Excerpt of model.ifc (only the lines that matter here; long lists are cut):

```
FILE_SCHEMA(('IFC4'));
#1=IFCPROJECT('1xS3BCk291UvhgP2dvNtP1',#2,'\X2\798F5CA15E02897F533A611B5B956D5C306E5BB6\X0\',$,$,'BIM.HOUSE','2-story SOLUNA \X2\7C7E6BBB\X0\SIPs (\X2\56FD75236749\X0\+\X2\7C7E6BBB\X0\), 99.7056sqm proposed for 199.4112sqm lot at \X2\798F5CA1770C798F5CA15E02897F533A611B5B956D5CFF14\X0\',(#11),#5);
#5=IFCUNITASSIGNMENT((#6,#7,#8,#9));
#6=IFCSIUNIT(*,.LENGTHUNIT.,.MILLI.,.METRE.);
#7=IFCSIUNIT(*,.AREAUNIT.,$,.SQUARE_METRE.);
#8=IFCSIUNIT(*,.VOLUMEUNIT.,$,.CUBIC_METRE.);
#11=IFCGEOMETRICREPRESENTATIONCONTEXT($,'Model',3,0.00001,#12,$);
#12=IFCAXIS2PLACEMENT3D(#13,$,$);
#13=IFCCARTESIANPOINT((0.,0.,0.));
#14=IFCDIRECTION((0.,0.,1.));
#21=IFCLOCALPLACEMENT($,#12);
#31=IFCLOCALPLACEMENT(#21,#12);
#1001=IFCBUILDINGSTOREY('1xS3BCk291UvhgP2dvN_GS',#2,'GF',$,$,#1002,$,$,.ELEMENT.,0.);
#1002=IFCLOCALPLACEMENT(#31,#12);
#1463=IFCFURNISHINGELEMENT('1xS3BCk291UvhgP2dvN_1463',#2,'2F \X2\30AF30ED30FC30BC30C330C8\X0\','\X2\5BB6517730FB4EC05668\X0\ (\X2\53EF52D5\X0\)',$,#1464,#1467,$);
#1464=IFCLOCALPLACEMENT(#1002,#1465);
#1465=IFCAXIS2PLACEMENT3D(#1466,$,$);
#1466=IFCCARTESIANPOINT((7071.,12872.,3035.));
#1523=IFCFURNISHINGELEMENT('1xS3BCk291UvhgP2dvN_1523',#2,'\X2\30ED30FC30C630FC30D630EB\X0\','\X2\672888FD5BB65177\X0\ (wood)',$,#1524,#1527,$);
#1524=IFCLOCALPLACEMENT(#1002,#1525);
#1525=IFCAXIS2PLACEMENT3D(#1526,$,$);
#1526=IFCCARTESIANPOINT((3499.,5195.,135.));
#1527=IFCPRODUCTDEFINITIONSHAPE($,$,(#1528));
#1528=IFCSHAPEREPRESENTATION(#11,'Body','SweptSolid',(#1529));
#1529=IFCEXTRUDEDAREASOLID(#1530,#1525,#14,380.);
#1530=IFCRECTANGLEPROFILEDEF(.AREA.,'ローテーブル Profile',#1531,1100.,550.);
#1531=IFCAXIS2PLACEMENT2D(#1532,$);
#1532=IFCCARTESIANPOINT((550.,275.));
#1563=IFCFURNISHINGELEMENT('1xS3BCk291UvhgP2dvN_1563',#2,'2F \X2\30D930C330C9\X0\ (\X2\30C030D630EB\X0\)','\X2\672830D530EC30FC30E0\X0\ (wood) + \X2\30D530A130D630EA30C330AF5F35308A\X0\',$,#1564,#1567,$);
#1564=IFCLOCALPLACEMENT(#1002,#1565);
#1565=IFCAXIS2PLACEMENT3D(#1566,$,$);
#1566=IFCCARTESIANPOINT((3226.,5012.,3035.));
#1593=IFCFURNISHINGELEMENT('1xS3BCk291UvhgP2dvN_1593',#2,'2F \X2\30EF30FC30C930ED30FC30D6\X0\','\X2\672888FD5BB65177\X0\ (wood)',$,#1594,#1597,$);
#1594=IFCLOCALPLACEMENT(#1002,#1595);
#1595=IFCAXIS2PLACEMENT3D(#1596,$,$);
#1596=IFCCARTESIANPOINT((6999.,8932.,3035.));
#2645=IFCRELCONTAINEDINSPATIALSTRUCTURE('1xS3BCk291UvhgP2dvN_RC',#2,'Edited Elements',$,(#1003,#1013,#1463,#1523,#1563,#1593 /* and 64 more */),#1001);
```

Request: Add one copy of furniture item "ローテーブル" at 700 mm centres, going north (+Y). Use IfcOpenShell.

```python
import numpy as np
import ifcopenshell
import ifcopenshell.api.geometry
import ifcopenshell.api.root
import ifcopenshell.util.element
import ifcopenshell.util.placement

model = ifcopenshell.open("model.ifc")


def reuse_history(source, copy):
    """copy_class also copies each property set's owner history, people and application; keep the originals."""
    for rel in copy.IsDefinedBy:
        if rel.is_a("IfcRelDefinesByProperties") and (history := rel.RelatingPropertyDefinition.OwnerHistory):
            rel.RelatingPropertyDefinition.OwnerHistory = source.OwnerHistory
            ifcopenshell.util.element.remove_deep2(model, history)


source = model.by_guid("1xS3BCk291UvhgP2dvN_1523")
base = ifcopenshell.util.placement.get_local_placement(source.ObjectPlacement)
step = np.array([0.0, 1.0, 0.0]) * 700.0

for i in range(1, 2):
    copy = ifcopenshell.api.root.copy_class(model, product=source)
    copy.Representation = ifcopenshell.util.element.copy_deep(
        model, source.Representation, exclude=["IfcGeometricRepresentationContext", "IfcRepresentationMap"]
    )
    reuse_history(source, copy)
    matrix = base.copy()
    matrix[:3, 3] += i * step
    print("added at", matrix[:3, 3].round(3) + 0.0)
    ifcopenshell.api.geometry.edit_object_placement(model, product=copy, matrix=matrix, is_si=False)

model.write("model_v2.ifc")
```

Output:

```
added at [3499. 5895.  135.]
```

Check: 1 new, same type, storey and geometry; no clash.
